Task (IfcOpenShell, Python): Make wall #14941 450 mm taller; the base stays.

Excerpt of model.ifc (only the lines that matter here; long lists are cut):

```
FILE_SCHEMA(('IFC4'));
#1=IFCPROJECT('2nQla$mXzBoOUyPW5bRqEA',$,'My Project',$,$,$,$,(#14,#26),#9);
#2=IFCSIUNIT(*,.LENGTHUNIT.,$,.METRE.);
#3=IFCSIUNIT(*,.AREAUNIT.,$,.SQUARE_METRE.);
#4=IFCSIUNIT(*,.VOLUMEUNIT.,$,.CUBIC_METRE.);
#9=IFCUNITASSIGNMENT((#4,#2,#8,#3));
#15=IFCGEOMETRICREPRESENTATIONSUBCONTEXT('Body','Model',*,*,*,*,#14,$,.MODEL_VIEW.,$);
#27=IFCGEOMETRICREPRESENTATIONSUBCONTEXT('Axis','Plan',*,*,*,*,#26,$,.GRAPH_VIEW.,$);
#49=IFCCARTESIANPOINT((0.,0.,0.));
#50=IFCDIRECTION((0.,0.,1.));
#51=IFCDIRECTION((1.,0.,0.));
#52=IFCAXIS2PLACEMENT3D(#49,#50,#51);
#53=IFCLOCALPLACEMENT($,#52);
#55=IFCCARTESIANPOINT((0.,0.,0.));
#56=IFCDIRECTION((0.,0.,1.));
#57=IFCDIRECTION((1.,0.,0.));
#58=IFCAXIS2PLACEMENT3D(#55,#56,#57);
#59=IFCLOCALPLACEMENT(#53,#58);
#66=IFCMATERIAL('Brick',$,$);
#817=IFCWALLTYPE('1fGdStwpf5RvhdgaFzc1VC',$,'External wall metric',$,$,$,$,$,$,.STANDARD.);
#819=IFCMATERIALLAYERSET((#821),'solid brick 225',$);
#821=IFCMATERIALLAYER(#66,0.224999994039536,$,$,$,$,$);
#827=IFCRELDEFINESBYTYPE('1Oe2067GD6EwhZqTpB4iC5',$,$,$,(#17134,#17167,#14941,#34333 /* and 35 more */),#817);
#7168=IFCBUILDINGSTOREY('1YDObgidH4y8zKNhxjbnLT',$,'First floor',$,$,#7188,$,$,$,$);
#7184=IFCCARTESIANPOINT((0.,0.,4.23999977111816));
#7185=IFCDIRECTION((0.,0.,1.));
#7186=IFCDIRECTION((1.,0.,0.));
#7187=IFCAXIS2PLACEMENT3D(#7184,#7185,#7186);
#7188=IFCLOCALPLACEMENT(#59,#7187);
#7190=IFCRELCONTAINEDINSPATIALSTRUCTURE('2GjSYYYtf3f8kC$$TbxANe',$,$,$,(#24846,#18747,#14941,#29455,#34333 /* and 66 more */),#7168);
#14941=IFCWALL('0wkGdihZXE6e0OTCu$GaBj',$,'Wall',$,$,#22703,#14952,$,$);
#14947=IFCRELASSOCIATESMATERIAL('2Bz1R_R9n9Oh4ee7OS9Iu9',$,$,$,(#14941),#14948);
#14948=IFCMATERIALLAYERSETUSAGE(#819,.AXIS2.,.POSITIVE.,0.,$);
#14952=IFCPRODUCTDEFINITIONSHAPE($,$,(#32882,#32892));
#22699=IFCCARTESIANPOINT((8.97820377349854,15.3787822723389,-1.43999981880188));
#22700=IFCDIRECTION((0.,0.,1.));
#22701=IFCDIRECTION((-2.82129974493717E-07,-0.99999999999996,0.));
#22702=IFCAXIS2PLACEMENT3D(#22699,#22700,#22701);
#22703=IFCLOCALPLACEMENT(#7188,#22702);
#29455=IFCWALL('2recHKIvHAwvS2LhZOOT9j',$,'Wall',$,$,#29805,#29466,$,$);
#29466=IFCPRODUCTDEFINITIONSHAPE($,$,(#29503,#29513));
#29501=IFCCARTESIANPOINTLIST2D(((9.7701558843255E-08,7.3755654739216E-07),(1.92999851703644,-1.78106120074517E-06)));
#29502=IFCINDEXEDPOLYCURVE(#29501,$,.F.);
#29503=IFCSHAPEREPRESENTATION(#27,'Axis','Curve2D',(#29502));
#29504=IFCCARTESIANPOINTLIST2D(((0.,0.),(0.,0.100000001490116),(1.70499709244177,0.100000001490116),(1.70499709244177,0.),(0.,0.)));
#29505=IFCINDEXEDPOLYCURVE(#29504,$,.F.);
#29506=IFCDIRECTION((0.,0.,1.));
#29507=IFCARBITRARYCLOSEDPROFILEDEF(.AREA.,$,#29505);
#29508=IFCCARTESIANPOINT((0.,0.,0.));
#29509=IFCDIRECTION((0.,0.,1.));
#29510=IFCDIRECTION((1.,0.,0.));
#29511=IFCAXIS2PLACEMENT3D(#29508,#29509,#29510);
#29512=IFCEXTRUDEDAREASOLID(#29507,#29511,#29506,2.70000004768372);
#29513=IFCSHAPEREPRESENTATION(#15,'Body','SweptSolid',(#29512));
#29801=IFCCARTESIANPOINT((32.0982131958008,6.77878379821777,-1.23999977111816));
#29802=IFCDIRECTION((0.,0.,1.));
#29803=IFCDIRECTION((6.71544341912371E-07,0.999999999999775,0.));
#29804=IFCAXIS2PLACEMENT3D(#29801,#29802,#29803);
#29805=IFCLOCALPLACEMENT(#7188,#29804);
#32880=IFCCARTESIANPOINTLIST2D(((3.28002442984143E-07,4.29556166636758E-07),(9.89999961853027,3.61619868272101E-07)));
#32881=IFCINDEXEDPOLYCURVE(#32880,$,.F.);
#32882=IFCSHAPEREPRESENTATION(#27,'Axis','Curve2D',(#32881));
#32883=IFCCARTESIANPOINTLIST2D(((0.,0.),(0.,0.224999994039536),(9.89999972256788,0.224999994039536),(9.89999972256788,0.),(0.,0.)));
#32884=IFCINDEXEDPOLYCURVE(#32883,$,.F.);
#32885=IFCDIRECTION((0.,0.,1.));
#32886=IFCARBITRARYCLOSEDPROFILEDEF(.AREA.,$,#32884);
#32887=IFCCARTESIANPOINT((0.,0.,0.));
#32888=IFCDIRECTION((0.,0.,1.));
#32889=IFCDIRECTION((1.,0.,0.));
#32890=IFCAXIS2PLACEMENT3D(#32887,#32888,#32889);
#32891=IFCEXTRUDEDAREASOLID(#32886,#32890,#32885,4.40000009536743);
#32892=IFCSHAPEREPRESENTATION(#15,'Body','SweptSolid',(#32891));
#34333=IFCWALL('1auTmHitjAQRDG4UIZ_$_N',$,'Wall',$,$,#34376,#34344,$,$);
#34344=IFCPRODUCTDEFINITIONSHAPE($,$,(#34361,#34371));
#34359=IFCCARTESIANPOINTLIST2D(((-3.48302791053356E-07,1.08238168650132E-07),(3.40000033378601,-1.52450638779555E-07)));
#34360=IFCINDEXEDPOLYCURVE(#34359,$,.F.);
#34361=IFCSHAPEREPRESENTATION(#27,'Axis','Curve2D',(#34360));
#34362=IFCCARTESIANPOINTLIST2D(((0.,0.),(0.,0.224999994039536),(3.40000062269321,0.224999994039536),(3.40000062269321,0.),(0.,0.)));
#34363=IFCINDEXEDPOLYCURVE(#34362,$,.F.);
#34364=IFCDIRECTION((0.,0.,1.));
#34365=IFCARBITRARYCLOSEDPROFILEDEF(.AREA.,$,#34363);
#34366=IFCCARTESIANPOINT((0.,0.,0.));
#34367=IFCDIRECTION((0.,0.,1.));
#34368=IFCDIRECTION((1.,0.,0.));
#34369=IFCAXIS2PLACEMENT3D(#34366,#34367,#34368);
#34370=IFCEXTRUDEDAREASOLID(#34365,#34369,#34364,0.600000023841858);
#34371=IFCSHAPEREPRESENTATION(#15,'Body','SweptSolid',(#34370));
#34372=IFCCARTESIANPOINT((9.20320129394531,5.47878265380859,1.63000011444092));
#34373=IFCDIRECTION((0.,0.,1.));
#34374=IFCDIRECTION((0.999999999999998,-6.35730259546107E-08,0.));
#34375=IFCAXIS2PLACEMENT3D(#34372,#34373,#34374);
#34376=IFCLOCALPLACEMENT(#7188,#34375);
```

```python
import ifcopenshell
import ifcopenshell.geom
import ifcopenshell.util.representation
import ifcopenshell.util.shape
import ifcopenshell.util.unit

model = ifcopenshell.open("model.ifc")
unit_scale = ifcopenshell.util.unit.calculate_unit_scale(model)
settings = ifcopenshell.geom.settings()


def volume(element):
    """Net volume in cubic metres, openings subtracted."""
    shape = ifcopenshell.geom.create_shape(settings, element)
    return ifcopenshell.util.shape.get_volume(shape.geometry)


wall = model.by_guid("0wkGdihZXE6e0OTCu$GaBj")
before = volume(wall)

body = ifcopenshell.util.representation.get_representation(wall, "Model", "Body")
solid = body.Items[0]
old_height = solid.Depth
solid.Depth += 0.45 / unit_scale
after = volume(wall)

print(f"height {old_height:g} -> {solid.Depth:g}, volume {before:.3f} -> {after:.3f} m3")

model.write("model_v2.ifc")
```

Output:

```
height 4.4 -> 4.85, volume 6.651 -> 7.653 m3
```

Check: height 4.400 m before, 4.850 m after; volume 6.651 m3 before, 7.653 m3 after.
